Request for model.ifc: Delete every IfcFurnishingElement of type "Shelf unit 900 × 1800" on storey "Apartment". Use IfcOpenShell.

First a look at what the model holds.

```python
import ifcopenshell
import ifcopenshell.util.element

model = ifcopenshell.open("model.ifc")
print(model.schema)
storey = next(s for s in model.by_type("IfcBuildingStorey") if s.Name == "Apartment")
furniture = [e for e in ifcopenshell.util.element.get_decomposition(storey) if e.is_a("IfcFurnishingElement")]
seen = {}
for e in furniture:
    element_type = ifcopenshell.util.element.get_type(e)
    name = element_type.Name if element_type not in (None, e) else None
    seen[name] = seen.get(name, 0) + 1
for name, count in sorted(seen.items(), key=str):
    print(count, "x", name)
```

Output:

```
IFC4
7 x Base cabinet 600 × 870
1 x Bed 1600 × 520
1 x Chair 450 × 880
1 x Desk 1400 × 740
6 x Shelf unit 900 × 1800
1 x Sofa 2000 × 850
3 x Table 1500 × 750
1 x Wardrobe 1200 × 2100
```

```python
import ifcopenshell
import ifcopenshell.api.root
import ifcopenshell.util.element

model = ifcopenshell.open("model.ifc")

storey = next(s for s in model.by_type("IfcBuildingStorey") if s.Name == "Apartment")
furniture = [e for e in ifcopenshell.util.element.get_decomposition(storey) if e.is_a("IfcFurnishingElement")]
targets = [e for e in furniture if (t := ifcopenshell.util.element.get_type(e)) not in (None, e) and t.Name == "Shelf unit 900 × 1800"]

for e in targets:
    ifcopenshell.api.root.remove_product(model, product=e)
print(len(targets), "removed")

model.write("model_rev.ifc")
```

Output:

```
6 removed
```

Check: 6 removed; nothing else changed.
